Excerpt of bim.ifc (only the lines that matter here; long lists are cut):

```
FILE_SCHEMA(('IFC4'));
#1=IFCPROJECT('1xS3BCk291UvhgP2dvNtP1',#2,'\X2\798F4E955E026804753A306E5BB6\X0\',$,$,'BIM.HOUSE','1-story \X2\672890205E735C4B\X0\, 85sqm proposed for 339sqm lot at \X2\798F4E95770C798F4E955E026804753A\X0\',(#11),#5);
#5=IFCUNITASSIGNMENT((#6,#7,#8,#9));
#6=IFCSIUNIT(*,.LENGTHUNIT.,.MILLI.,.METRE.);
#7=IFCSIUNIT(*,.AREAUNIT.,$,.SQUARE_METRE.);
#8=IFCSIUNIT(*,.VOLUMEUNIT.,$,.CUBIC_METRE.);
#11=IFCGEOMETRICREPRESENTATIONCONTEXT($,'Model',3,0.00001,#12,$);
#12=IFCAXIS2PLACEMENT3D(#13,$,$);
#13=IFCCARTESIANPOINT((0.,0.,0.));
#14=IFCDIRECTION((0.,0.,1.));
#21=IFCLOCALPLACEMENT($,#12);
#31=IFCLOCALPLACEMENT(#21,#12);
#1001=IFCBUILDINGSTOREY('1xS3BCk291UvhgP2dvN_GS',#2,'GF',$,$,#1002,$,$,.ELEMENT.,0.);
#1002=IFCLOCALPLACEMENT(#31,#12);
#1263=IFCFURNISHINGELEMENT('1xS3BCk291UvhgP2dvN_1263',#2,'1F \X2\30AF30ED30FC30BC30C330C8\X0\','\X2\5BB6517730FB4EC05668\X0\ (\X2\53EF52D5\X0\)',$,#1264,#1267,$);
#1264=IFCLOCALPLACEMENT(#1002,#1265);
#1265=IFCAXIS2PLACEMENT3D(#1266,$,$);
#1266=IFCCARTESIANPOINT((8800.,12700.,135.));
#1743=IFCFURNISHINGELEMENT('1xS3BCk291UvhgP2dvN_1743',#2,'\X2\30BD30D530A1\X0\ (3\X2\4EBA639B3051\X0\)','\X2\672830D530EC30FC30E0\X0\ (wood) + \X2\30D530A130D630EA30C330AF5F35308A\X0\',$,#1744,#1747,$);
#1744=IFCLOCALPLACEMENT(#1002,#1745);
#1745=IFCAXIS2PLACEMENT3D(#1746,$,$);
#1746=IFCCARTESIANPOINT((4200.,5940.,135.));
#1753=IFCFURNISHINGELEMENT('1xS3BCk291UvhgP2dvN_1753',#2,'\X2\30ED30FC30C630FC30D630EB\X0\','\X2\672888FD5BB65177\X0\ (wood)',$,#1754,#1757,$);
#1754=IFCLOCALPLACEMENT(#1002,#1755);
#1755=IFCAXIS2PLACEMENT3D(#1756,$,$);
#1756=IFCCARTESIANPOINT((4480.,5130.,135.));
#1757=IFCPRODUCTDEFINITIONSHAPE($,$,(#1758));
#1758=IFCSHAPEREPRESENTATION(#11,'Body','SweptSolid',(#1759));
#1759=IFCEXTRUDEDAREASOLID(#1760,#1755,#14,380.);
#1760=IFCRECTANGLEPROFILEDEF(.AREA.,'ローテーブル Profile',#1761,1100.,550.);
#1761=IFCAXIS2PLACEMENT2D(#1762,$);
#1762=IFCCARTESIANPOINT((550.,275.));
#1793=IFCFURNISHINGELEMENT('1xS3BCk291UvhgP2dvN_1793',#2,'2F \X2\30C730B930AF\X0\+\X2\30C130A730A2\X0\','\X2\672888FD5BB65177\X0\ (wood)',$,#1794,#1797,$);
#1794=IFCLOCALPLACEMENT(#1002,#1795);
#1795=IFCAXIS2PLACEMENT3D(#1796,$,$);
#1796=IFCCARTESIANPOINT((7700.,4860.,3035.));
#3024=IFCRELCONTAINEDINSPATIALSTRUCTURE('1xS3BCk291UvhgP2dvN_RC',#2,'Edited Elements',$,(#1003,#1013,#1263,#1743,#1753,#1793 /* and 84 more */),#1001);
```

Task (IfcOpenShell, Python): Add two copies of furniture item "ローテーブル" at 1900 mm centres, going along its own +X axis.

```python
import ifcopenshell
import ifcopenshell.api.geometry
import ifcopenshell.api.root
import ifcopenshell.util.element
import ifcopenshell.util.placement
import ifcopenshell.util.unit

model = ifcopenshell.open("bim.ifc")
unit_scale = ifcopenshell.util.unit.calculate_unit_scale(model)


def reuse_history(source, copy):
    """copy_class also copies each property set's owner history, people and application; keep the originals."""
    for rel in copy.IsDefinedBy:
        if rel.is_a("IfcRelDefinesByProperties") and (history := rel.RelatingPropertyDefinition.OwnerHistory):
            rel.RelatingPropertyDefinition.OwnerHistory = source.OwnerHistory
            ifcopenshell.util.element.remove_deep2(model, history)


source = model.by_guid("1xS3BCk291UvhgP2dvN_1753")
base = ifcopenshell.util.placement.get_local_placement(source.ObjectPlacement)
step = base[:3, 0] * 1.9 / unit_scale

for i in range(1, 3):
    copy = ifcopenshell.api.root.copy_class(model, product=source)
    copy.Representation = ifcopenshell.util.element.copy_deep(
        model, source.Representation, exclude=["IfcGeometricRepresentationContext", "IfcRepresentationMap"]
    )
    reuse_history(source, copy)
    matrix = base.copy()
    matrix[:3, 3] += i * step
    print("added at", matrix[:3, 3].round(3) + 0.0)
    ifcopenshell.api.geometry.edit_object_placement(model, product=copy, matrix=matrix, is_si=False)

model.write("bim_rev.ifc")
```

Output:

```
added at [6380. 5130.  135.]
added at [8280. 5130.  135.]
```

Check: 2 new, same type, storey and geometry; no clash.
